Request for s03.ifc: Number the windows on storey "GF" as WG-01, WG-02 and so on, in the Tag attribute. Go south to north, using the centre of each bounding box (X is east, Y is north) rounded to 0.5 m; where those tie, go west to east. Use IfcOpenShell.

First a look at what the model holds.

```python
import ifcopenshell
import ifcopenshell.util.element
import ifcopenshell.util.placement

model = ifcopenshell.open("s03.ifc")
print(model.schema)
storey = next(s for s in model.by_type("IfcBuildingStorey") if s.Name == "GF")
windows = [e for e in ifcopenshell.util.element.get_decomposition(storey) if e.is_a("IfcWindow")]
for e in sorted(windows, key=lambda e: e.id()):
    origin = ifcopenshell.util.placement.get_local_placement(e.ObjectPlacement)[:3, 3]
    print(e.id(), e.Tag, e.Name, origin.round(2) + 0.0, sep=" | ")
```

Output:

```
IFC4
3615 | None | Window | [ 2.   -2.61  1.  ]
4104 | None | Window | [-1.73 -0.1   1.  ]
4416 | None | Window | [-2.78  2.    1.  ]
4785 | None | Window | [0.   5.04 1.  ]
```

```python
import ifcopenshell
import ifcopenshell.geom
import ifcopenshell.util.element
import ifcopenshell.util.shape

model = ifcopenshell.open("s03.ifc")
settings = ifcopenshell.geom.settings()
settings.set("use-world-coords", True)


def centre(element):
    shape = ifcopenshell.geom.create_shape(settings, element)
    return ifcopenshell.util.shape.get_bbox_centroid(shape.geometry)


storey = next(s for s in model.by_type("IfcBuildingStorey") if s.Name == "GF")
windows = [e for e in ifcopenshell.util.element.get_decomposition(storey) if e.is_a("IfcWindow")]

# Insertion points can sit at a corner or the storey origin, so sort by the geometry (in metres).
centres = {e: centre(e) for e in windows}
windows.sort(key=lambda e: (round(centres[e][1] / 0.5), centres[e][0]))

for i, e in enumerate(windows, start=1):
    number = f"WG-{i:02d}"
    e.Tag = number
    print(e.id(), number)

model.write("s03_edited.ifc")
```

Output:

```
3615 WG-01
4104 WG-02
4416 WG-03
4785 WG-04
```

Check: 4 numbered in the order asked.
